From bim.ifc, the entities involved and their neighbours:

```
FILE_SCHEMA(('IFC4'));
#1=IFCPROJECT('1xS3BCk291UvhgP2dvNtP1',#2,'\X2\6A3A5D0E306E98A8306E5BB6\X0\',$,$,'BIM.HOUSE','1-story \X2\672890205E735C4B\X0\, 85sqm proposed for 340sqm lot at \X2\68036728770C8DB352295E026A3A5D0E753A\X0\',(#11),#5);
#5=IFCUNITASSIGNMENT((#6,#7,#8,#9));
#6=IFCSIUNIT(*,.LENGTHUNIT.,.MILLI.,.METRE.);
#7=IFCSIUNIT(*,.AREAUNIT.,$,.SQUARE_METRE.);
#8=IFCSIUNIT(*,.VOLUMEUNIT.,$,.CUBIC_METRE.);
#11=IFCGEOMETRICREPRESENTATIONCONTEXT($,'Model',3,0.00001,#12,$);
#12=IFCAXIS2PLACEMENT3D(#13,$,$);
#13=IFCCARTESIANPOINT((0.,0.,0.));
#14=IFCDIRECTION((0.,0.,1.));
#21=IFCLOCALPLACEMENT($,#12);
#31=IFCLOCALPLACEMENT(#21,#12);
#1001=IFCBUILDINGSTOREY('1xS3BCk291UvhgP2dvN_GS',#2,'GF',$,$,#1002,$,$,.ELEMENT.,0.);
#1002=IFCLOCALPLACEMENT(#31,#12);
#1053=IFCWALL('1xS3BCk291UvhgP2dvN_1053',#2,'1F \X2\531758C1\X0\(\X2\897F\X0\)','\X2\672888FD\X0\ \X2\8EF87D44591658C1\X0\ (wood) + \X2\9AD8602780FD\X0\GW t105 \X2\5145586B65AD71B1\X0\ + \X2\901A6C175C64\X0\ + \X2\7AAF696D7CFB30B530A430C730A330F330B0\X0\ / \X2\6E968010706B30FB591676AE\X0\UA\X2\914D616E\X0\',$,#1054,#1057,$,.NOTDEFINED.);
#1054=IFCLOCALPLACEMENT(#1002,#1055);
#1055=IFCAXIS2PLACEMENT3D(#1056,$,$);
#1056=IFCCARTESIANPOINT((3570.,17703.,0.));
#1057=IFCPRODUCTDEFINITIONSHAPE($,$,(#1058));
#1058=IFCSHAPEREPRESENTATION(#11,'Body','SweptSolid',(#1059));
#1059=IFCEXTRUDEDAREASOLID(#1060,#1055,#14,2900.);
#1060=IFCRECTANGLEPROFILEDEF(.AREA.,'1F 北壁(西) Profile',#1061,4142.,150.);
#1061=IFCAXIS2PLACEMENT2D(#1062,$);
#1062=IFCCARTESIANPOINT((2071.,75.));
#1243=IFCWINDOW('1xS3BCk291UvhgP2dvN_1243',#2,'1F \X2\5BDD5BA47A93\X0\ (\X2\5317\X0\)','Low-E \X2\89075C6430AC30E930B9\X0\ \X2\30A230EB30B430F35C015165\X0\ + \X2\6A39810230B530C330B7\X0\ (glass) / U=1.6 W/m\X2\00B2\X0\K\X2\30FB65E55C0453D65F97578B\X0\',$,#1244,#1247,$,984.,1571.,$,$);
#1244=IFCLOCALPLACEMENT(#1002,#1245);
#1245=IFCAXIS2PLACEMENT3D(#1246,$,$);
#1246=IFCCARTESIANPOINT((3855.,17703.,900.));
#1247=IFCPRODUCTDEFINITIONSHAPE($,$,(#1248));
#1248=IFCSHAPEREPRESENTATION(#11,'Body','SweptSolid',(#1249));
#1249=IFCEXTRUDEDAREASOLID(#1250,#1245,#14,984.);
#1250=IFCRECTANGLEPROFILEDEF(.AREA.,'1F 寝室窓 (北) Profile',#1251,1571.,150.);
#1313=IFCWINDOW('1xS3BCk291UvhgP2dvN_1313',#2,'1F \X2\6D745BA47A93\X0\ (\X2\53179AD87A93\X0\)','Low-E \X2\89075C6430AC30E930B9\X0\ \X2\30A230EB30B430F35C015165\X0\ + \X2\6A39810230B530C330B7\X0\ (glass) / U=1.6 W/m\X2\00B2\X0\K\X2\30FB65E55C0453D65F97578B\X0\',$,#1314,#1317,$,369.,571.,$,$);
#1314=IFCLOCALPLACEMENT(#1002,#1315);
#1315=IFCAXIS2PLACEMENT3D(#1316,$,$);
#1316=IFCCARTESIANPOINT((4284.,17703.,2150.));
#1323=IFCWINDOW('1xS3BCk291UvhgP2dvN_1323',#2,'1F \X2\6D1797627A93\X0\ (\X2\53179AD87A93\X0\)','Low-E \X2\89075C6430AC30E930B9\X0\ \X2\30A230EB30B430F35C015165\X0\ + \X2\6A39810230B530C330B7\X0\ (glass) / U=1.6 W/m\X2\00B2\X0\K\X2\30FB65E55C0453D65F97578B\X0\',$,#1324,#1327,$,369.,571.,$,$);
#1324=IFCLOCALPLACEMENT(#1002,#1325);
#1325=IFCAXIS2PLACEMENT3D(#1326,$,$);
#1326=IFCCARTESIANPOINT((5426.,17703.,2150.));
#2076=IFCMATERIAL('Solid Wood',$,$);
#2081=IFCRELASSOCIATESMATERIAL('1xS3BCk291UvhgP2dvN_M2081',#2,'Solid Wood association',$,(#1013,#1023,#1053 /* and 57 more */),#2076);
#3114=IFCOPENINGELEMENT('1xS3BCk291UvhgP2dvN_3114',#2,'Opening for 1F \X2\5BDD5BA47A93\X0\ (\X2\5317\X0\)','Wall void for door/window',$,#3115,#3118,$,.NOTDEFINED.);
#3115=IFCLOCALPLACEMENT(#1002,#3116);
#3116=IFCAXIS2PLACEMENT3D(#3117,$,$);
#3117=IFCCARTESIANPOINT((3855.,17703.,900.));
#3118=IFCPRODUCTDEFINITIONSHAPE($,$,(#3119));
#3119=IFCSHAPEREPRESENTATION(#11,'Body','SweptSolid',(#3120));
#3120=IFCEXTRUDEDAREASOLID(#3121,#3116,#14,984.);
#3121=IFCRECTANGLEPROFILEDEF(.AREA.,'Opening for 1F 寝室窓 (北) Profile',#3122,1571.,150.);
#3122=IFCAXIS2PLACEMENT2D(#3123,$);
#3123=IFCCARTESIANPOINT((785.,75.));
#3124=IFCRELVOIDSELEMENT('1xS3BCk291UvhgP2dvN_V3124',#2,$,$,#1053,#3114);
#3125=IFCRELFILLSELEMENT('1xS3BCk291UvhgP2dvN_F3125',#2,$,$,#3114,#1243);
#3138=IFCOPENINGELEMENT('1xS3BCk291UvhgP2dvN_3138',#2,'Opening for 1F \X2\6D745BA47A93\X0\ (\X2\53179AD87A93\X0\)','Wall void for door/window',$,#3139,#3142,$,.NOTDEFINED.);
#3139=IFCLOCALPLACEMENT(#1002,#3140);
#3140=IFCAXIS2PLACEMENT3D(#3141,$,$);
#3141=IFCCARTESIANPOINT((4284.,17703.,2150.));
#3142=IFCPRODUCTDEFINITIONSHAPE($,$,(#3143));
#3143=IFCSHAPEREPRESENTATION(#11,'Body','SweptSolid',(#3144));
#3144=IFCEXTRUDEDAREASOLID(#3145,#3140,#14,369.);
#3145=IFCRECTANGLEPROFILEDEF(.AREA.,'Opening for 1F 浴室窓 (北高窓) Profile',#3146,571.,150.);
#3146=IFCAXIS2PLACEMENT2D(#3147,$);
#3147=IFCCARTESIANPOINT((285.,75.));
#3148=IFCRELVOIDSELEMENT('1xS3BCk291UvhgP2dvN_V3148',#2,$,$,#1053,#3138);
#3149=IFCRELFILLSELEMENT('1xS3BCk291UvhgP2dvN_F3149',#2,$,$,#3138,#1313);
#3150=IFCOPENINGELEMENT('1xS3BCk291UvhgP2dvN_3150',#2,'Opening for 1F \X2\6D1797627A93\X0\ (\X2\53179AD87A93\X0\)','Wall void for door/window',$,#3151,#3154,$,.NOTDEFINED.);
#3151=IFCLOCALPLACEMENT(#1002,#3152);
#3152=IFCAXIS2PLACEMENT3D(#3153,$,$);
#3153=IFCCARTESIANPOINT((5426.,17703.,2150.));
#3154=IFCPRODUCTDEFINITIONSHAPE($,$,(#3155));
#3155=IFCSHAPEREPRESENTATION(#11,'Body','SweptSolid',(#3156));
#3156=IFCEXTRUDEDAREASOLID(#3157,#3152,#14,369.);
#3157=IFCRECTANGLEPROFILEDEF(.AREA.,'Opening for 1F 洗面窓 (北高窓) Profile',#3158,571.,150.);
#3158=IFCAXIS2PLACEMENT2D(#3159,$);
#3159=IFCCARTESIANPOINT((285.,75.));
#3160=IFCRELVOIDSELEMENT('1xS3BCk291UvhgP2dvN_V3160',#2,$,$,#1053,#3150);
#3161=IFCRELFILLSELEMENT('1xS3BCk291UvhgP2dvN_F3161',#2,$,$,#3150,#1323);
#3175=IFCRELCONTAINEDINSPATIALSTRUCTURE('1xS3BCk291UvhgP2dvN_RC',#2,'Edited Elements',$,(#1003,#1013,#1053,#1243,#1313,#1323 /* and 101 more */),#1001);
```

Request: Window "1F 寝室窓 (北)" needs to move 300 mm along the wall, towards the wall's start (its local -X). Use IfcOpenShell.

```python
import ifcopenshell
import ifcopenshell.api.geometry
import ifcopenshell.util.placement
import ifcopenshell.util.unit

model = ifcopenshell.open("bim.ifc")
unit_scale = ifcopenshell.util.unit.calculate_unit_scale(model)

window = model.by_guid("1xS3BCk291UvhgP2dvN_1243")
opening = window.FillsVoids[0].RelatingOpeningElement
wall = opening.VoidsElements[0].RelatingBuildingElement

wall_matrix = ifcopenshell.util.placement.get_local_placement(wall.ObjectPlacement)
shift = wall_matrix[:3, 0] * -0.3 / unit_scale
before = ifcopenshell.util.placement.get_local_placement(window.ObjectPlacement)[:3, 3].copy()

# The window is not placed relative to its opening, so move both.
for product in (opening, window):
    matrix = ifcopenshell.util.placement.get_local_placement(product.ObjectPlacement)
    matrix[:3, 3] += shift
    ifcopenshell.api.geometry.edit_object_placement(model, product=product, matrix=matrix, is_si=False)

after = ifcopenshell.util.placement.get_local_placement(window.ObjectPlacement)[:3, 3]
print("window moved by", (after - before).round(3) + 0.0)

model.write("bim_rev.ifc")
```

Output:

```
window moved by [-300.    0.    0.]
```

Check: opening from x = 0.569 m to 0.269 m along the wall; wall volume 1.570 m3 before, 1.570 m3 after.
